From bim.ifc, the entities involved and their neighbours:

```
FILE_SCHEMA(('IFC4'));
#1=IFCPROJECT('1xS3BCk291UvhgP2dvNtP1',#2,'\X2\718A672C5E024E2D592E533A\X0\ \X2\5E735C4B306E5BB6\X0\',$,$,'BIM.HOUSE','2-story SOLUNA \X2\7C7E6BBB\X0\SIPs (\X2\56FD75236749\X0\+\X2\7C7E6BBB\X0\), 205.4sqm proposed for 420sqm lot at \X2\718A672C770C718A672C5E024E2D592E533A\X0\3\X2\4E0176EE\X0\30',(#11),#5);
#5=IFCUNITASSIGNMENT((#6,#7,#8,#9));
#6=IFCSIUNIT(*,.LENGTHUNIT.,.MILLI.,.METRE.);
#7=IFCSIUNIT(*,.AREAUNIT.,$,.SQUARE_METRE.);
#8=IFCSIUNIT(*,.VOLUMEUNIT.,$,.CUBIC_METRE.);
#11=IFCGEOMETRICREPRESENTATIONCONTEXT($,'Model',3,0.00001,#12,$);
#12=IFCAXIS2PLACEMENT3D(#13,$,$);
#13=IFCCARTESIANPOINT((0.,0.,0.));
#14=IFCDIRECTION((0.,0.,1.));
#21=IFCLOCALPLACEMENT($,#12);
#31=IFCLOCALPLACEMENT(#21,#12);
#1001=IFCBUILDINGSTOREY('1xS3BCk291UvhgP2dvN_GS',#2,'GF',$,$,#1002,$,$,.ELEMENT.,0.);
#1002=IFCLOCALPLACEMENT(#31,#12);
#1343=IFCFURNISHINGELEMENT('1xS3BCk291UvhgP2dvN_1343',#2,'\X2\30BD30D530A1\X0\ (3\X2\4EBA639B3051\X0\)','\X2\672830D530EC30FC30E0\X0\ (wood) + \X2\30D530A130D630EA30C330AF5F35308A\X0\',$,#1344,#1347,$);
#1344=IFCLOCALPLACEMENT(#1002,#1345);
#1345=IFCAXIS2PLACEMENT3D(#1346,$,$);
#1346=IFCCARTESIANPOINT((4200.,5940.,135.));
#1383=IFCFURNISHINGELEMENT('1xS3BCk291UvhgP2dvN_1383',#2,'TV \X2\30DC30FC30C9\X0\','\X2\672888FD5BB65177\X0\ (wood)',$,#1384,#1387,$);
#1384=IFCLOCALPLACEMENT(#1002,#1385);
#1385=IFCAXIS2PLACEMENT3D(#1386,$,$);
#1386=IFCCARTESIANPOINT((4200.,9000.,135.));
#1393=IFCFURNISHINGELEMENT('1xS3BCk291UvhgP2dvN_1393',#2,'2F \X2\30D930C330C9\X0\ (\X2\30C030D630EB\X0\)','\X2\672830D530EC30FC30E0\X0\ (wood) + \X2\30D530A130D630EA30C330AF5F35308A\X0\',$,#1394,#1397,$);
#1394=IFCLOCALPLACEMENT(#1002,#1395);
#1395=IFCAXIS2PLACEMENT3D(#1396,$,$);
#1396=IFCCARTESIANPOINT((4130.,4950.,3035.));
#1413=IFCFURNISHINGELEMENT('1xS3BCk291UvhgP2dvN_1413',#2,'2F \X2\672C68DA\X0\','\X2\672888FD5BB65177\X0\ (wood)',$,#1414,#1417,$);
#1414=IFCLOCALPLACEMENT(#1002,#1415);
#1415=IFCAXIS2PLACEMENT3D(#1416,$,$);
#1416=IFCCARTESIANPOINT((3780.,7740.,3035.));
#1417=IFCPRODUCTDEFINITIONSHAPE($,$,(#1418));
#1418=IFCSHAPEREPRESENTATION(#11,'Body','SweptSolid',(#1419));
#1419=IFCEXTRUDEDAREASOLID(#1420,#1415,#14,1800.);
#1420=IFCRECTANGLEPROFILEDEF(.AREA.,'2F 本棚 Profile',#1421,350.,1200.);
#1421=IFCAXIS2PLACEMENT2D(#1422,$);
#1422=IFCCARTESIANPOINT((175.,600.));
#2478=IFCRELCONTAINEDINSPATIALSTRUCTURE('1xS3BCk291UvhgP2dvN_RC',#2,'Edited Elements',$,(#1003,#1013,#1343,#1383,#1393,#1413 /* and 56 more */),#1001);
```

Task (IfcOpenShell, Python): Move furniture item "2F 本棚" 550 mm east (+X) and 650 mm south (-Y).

```python
import ifcopenshell
import ifcopenshell.api.geometry
import ifcopenshell.util.placement

model = ifcopenshell.open("bim.ifc")

item = model.by_guid("1xS3BCk291UvhgP2dvN_1413")
matrix = ifcopenshell.util.placement.get_local_placement(item.ObjectPlacement)
matrix[0, 3] += 550.0
matrix[1, 3] -= 650.0
ifcopenshell.api.geometry.edit_object_placement(model, product=item, matrix=matrix, is_si=False)

print(ifcopenshell.util.placement.get_local_placement(item.ObjectPlacement).round(3) + 0.0)

model.write("bim_updated.ifc")
```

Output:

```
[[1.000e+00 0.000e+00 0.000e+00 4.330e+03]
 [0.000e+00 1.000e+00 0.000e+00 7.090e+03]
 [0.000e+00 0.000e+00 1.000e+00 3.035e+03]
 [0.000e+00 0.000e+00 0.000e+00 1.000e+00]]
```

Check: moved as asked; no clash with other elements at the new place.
